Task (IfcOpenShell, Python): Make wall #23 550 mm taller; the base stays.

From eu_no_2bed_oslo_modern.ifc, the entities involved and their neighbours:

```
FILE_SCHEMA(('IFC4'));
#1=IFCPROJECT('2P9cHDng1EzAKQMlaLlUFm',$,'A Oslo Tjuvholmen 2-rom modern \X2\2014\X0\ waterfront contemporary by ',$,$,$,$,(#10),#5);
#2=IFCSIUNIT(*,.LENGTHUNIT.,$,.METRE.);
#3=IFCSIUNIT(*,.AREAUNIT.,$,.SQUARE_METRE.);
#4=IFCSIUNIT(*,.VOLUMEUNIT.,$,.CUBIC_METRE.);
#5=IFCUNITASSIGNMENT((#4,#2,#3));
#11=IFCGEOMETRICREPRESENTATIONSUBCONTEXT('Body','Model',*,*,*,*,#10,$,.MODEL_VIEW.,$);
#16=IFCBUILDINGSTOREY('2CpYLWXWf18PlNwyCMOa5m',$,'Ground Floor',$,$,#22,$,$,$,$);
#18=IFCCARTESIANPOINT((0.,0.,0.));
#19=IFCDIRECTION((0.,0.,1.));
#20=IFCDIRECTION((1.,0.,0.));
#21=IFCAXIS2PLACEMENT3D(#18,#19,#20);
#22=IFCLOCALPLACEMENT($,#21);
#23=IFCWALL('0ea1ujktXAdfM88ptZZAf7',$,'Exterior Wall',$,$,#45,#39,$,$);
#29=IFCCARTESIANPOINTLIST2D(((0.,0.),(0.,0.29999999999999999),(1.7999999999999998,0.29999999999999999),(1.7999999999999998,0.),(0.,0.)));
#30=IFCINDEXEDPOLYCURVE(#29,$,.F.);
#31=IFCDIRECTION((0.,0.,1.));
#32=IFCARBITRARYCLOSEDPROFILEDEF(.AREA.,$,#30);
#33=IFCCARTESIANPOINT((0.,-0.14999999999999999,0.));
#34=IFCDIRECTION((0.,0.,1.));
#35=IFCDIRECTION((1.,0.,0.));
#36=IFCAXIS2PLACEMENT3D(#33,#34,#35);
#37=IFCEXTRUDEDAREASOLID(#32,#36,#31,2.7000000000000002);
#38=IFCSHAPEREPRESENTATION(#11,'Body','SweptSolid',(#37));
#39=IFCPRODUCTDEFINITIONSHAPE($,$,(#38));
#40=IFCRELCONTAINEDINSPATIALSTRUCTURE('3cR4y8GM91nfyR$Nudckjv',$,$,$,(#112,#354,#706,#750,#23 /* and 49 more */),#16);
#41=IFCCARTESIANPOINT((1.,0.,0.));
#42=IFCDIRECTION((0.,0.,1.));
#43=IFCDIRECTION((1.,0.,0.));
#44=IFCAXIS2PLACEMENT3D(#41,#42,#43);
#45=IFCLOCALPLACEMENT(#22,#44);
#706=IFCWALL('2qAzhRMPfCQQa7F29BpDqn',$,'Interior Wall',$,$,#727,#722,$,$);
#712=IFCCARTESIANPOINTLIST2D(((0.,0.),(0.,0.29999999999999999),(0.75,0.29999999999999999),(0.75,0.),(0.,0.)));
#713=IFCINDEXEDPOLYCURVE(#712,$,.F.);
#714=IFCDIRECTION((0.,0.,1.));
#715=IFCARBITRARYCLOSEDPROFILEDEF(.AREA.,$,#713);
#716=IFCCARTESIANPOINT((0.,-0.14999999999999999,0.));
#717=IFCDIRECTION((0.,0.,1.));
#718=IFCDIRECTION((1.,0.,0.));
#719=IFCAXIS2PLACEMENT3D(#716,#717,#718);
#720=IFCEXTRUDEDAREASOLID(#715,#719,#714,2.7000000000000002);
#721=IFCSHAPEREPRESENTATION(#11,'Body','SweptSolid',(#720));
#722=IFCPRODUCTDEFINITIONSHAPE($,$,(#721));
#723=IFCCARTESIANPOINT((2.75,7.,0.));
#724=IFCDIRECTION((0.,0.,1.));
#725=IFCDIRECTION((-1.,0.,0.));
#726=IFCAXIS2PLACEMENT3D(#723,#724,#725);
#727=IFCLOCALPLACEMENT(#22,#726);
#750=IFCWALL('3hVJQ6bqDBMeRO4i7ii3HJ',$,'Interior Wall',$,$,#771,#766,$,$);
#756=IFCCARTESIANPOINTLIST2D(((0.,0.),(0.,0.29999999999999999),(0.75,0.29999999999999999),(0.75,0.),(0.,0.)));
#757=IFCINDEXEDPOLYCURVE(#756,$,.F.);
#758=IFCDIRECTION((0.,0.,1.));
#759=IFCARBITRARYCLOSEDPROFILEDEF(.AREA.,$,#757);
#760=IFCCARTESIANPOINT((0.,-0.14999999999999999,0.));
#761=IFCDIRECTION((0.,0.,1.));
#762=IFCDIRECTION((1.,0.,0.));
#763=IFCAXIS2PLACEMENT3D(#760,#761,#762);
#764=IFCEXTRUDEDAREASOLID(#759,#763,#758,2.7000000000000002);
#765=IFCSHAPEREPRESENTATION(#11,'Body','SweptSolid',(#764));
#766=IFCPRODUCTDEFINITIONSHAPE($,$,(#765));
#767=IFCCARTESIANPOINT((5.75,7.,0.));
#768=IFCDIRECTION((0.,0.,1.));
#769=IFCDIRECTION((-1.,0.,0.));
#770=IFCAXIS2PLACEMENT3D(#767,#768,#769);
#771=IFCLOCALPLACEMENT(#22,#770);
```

```python
import ifcopenshell
import ifcopenshell.geom
import ifcopenshell.util.representation
import ifcopenshell.util.shape
import ifcopenshell.util.unit

model = ifcopenshell.open("eu_no_2bed_oslo_modern.ifc")
unit_scale = ifcopenshell.util.unit.calculate_unit_scale(model)
settings = ifcopenshell.geom.settings()


def volume(element):
    """Net volume in cubic metres, openings subtracted."""
    shape = ifcopenshell.geom.create_shape(settings, element)
    return ifcopenshell.util.shape.get_volume(shape.geometry)


wall = model.by_guid("0ea1ujktXAdfM88ptZZAf7")
before = volume(wall)

body = ifcopenshell.util.representation.get_representation(wall, "Model", "Body")
solid = body.Items[0]
old_height = solid.Depth
solid.Depth += 0.55 / unit_scale
after = volume(wall)

print(f"height {old_height:g} -> {solid.Depth:g}, volume {before:.3f} -> {after:.3f} m3")

model.write("eu_no_2bed_oslo_modern_v2.ifc")
```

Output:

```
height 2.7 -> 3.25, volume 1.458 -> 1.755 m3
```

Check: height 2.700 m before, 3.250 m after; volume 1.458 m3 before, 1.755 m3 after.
